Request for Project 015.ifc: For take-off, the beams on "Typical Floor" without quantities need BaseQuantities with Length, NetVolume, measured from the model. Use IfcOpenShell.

First a look at what the model holds.

```python
import ifcopenshell
import ifcopenshell.util.element
import ifcopenshell.util.unit

model = ifcopenshell.open("Project 015.ifc")
print(model.schema)
for unit_type in ("LENGTHUNIT", "AREAUNIT", "VOLUMEUNIT"):
    print(unit_type, ifcopenshell.util.unit.calculate_unit_scale(model, unit_type))
storey = next(s for s in model.by_type("IfcBuildingStorey") if s.Name == "Typical Floor")
beams = [e for e in ifcopenshell.util.element.get_decomposition(storey) if e.is_a("IfcBeam")]
for e in sorted(beams, key=lambda e: e.id()):
    print(e.id(), e.is_a(), e.Name, list(ifcopenshell.util.element.get_psets(e, qtos_only=True)), sep=" | ")
```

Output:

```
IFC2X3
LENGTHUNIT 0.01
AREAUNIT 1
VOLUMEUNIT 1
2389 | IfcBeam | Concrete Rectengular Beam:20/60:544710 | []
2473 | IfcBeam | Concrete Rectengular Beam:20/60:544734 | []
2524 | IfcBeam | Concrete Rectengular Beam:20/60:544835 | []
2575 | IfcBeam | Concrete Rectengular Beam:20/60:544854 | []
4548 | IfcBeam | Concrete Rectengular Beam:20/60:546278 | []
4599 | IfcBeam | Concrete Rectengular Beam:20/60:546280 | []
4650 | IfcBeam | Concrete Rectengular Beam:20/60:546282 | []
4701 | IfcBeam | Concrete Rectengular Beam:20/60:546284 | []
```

```python
import ifcopenshell
import ifcopenshell.api.pset
import ifcopenshell.geom
import ifcopenshell.util.element
import ifcopenshell.util.shape
import ifcopenshell.util.unit

model = ifcopenshell.open("Project 015.ifc")
unit_scale = ifcopenshell.util.unit.calculate_unit_scale(model)
volume_scale = ifcopenshell.util.unit.calculate_unit_scale(model, "VOLUMEUNIT")
settings = ifcopenshell.geom.settings()

storey = next(s for s in model.by_type("IfcBuildingStorey") if s.Name == "Typical Floor")
beams = [e for e in ifcopenshell.util.element.get_decomposition(storey) if e.is_a("IfcBeam")]

for e in sorted(beams, key=lambda e: e.id()):
    if ifcopenshell.util.element.get_psets(e, qtos_only=True, should_inherit=False):
        continue
    # Geometry comes back in metres, in the element's own axes.
    shape = ifcopenshell.geom.create_shape(settings, e)
    values = {
        "Length": ifcopenshell.util.shape.get_max_xyz(shape.geometry) / unit_scale,
        "NetVolume": ifcopenshell.util.shape.get_volume(shape.geometry) / volume_scale,
    }
    qto = ifcopenshell.api.pset.add_qto(model, product=e, name="BaseQuantities")
    ifcopenshell.api.pset.edit_qto(model, qto=qto, properties=values)
    print(e.id(), {k: round(v, 3) for k, v in values.items()})

model.write("Project 015_updated.ifc")
```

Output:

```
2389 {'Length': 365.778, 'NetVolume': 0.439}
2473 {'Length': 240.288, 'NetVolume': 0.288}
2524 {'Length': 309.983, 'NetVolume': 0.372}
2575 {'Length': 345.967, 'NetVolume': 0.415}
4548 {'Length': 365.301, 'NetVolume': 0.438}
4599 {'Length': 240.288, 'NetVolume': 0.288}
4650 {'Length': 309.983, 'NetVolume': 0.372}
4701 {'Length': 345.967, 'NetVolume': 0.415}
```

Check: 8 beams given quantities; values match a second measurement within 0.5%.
